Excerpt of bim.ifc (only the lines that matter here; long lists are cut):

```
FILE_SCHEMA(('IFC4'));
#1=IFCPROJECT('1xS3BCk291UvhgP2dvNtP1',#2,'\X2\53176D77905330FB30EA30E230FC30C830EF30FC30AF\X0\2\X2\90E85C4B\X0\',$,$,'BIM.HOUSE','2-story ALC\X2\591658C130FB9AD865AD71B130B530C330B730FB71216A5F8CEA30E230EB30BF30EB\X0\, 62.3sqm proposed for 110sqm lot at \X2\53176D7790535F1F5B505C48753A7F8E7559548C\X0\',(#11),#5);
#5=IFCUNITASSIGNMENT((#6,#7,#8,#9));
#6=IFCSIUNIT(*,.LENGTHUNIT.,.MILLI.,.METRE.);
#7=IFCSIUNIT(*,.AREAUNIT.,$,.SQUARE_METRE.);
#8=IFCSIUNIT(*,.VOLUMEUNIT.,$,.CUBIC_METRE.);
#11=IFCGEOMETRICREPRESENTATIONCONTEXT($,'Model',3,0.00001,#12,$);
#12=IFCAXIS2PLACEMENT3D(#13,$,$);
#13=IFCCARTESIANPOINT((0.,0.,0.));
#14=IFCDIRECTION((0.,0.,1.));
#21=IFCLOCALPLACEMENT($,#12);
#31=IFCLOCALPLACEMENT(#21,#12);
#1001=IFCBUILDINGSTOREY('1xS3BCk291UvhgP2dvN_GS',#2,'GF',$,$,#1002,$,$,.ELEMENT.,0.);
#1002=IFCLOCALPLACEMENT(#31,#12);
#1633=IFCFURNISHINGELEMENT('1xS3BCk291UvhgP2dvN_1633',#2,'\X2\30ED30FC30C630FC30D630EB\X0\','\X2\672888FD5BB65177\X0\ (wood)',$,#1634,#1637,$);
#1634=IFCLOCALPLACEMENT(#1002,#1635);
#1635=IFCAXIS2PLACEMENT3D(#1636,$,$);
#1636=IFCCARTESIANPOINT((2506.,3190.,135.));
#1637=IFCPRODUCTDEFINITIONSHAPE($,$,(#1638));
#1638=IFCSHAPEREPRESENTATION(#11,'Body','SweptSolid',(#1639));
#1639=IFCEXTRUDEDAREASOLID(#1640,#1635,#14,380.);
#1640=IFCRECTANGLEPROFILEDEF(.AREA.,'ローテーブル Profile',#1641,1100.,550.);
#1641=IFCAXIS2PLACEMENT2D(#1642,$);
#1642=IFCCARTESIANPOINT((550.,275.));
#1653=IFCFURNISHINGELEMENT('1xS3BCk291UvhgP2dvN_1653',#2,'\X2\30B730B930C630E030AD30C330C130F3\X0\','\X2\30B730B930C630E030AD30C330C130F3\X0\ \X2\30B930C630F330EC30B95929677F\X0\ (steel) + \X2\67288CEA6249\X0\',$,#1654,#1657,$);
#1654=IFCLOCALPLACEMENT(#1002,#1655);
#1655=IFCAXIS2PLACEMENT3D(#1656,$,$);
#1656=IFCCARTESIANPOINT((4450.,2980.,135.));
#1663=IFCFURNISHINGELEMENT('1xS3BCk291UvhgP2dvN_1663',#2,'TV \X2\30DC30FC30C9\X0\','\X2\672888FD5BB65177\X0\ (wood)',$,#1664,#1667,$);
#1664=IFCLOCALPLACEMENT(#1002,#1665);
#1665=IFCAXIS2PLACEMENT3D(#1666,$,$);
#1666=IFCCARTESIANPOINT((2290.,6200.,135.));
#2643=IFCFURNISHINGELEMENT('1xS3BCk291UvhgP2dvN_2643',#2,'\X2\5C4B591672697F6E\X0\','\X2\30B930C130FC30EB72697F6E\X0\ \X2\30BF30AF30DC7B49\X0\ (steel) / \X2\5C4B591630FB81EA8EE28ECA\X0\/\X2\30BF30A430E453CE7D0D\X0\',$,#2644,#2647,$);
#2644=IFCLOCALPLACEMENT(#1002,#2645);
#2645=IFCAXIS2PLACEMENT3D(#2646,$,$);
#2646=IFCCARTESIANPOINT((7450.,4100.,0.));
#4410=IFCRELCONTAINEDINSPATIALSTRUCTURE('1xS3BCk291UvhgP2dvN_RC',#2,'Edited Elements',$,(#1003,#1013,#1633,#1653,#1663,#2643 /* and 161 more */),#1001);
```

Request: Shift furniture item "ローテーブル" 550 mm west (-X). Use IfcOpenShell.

```python
import ifcopenshell
import ifcopenshell.api.geometry
import ifcopenshell.util.placement

model = ifcopenshell.open("bim.ifc")

item = model.by_id(1633)
matrix = ifcopenshell.util.placement.get_local_placement(item.ObjectPlacement)
matrix[0, 3] -= 550.0
ifcopenshell.api.geometry.edit_object_placement(model, product=item, matrix=matrix, is_si=False)

print(ifcopenshell.util.placement.get_local_placement(item.ObjectPlacement).round(3) + 0.0)

model.write("bim_edited.ifc")
```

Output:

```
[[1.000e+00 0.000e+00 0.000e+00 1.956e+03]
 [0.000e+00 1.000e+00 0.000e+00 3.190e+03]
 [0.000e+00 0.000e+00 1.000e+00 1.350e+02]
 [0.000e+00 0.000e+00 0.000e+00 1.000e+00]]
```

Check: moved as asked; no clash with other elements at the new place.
